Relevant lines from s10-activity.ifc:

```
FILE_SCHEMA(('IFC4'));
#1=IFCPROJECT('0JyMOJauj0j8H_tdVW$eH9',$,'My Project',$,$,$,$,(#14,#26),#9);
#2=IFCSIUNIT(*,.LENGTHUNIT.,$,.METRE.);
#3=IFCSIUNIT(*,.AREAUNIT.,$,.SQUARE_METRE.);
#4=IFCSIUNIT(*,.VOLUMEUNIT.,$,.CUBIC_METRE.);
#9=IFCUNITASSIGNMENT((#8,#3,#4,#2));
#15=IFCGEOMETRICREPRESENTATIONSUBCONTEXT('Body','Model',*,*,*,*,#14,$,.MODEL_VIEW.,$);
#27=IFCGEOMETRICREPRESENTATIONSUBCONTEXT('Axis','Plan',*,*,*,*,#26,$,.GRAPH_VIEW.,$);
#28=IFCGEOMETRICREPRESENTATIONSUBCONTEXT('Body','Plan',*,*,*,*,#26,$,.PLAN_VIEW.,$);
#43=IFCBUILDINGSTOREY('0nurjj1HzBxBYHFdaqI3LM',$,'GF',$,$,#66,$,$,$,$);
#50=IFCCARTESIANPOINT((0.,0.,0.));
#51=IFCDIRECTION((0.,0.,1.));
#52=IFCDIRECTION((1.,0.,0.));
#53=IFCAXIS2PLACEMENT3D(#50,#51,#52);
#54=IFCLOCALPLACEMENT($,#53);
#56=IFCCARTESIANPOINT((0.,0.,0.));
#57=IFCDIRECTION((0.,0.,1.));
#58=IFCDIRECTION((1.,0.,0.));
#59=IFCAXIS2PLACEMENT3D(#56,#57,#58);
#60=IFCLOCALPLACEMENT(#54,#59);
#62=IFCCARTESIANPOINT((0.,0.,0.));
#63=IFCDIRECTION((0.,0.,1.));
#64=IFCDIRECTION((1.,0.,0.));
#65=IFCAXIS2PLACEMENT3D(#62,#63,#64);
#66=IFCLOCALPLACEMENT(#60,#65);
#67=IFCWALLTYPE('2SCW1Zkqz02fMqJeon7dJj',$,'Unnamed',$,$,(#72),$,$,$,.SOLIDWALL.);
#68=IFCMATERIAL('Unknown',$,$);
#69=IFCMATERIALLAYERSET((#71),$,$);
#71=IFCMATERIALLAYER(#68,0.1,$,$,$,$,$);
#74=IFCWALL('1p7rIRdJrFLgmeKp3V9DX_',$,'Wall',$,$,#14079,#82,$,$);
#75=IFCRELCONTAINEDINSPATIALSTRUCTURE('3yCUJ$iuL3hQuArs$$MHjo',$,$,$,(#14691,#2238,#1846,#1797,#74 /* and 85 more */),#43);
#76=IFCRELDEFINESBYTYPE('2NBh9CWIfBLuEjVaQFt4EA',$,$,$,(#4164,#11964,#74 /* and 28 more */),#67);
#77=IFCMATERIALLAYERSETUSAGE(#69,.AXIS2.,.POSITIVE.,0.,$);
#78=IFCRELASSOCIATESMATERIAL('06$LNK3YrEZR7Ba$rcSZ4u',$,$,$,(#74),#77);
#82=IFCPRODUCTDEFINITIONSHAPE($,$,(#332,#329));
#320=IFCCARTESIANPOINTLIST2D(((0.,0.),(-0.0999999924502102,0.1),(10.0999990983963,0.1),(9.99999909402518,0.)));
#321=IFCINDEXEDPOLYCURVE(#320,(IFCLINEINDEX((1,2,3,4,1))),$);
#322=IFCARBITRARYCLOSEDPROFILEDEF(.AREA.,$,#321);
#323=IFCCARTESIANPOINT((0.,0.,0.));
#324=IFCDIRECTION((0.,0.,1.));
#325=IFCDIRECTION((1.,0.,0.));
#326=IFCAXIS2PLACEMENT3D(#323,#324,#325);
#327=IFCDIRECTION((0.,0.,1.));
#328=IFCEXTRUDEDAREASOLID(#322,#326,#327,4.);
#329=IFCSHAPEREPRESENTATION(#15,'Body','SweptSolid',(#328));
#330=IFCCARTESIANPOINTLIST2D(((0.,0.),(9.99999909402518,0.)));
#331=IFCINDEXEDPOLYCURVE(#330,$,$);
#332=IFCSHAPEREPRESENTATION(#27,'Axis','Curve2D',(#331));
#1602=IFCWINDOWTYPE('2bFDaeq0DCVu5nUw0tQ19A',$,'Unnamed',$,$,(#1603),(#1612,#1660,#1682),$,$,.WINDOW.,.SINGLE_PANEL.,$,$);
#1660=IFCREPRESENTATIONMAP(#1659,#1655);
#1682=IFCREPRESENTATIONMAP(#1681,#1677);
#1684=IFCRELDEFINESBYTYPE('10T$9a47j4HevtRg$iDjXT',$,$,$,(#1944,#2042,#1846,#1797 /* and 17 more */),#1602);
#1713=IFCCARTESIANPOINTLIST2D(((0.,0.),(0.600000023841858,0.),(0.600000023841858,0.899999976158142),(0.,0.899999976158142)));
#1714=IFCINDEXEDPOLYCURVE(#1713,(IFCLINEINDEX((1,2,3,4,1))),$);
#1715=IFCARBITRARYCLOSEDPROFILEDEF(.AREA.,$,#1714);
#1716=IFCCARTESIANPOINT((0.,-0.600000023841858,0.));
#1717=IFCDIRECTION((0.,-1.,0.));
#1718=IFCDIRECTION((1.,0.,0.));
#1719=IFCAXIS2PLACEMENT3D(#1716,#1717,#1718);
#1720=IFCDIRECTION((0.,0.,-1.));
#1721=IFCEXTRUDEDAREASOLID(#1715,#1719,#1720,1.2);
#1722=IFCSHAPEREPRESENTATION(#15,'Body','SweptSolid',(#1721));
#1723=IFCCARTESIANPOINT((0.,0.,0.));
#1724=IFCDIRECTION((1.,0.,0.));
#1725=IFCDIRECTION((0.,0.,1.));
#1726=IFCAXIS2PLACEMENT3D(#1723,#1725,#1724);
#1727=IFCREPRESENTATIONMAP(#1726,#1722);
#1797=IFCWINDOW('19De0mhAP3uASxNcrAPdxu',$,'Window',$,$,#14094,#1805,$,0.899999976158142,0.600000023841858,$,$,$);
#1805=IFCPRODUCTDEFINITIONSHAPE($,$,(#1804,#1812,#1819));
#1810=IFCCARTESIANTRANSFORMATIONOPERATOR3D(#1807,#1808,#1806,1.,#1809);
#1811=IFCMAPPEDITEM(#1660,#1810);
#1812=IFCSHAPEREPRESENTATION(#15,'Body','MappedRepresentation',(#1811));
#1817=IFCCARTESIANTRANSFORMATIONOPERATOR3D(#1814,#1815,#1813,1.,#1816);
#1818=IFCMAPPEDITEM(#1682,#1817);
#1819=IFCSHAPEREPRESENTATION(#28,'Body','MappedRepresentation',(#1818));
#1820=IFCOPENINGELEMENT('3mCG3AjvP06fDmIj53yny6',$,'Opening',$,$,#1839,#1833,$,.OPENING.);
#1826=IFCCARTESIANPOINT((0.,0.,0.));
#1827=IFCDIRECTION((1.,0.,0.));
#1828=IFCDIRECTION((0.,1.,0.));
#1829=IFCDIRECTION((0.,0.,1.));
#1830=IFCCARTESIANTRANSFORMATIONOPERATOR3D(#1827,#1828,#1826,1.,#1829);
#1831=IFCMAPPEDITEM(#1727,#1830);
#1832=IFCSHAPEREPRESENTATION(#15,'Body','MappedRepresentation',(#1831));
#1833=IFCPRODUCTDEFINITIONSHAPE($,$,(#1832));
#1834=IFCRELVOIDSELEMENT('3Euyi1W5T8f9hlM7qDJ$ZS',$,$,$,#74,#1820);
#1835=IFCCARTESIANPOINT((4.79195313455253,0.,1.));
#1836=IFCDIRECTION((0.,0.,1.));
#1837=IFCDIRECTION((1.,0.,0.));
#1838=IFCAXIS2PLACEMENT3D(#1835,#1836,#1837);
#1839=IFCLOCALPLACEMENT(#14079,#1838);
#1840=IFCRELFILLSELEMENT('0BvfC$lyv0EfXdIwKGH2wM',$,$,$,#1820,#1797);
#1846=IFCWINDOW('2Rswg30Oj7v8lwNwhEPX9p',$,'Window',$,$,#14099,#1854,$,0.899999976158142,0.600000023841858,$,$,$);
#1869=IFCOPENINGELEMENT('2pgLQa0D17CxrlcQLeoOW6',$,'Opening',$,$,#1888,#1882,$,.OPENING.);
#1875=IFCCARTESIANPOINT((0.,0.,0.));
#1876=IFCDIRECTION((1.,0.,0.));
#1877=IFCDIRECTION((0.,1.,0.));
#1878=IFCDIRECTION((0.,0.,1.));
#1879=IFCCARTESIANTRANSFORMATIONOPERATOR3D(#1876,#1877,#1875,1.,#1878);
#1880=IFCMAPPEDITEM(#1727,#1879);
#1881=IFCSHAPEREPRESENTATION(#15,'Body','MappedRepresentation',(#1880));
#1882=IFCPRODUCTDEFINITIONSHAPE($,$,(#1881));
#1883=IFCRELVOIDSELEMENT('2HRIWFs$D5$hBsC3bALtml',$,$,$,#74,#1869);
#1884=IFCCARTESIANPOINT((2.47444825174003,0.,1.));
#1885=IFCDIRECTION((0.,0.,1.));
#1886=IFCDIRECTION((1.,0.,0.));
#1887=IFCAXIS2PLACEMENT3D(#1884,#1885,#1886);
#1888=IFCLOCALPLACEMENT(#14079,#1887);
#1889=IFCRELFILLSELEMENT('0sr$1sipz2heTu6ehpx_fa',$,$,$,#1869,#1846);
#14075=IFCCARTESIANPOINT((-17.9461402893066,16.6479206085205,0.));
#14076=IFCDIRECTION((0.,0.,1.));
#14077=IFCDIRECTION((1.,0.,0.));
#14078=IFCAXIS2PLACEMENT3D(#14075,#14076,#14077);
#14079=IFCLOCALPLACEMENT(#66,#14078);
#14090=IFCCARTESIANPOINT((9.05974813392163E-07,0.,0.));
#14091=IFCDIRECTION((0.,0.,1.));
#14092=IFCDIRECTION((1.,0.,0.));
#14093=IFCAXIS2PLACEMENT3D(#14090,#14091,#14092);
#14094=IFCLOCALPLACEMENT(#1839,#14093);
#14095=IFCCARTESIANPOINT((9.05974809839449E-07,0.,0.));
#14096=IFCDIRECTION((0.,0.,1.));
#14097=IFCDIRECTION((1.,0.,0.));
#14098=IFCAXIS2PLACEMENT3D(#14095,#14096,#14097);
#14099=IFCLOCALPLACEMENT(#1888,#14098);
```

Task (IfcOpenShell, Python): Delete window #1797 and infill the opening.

```python
import ifcopenshell
import ifcopenshell.api.feature
import ifcopenshell.api.root
import ifcopenshell.geom
import ifcopenshell.util.shape

model = ifcopenshell.open("s10-activity.ifc")
settings = ifcopenshell.geom.settings()


def volume(element):
    """Net volume in cubic metres, openings subtracted."""
    shape = ifcopenshell.geom.create_shape(settings, element)
    return ifcopenshell.util.shape.get_volume(shape.geometry)


window = model.by_id(1797)
opening = window.FillsVoids[0].RelatingOpeningElement
wall = opening.VoidsElements[0].RelatingBuildingElement
before = volume(wall)

ifcopenshell.api.root.remove_product(model, product=window)
ifcopenshell.api.feature.remove_feature(model, feature=opening)

after = volume(wall)

print(f"wall volume {before:.3f} -> {after:.3f} m3")

model.write("s10-activity_rev.ifc")
```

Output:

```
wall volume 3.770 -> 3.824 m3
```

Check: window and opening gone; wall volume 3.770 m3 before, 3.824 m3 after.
